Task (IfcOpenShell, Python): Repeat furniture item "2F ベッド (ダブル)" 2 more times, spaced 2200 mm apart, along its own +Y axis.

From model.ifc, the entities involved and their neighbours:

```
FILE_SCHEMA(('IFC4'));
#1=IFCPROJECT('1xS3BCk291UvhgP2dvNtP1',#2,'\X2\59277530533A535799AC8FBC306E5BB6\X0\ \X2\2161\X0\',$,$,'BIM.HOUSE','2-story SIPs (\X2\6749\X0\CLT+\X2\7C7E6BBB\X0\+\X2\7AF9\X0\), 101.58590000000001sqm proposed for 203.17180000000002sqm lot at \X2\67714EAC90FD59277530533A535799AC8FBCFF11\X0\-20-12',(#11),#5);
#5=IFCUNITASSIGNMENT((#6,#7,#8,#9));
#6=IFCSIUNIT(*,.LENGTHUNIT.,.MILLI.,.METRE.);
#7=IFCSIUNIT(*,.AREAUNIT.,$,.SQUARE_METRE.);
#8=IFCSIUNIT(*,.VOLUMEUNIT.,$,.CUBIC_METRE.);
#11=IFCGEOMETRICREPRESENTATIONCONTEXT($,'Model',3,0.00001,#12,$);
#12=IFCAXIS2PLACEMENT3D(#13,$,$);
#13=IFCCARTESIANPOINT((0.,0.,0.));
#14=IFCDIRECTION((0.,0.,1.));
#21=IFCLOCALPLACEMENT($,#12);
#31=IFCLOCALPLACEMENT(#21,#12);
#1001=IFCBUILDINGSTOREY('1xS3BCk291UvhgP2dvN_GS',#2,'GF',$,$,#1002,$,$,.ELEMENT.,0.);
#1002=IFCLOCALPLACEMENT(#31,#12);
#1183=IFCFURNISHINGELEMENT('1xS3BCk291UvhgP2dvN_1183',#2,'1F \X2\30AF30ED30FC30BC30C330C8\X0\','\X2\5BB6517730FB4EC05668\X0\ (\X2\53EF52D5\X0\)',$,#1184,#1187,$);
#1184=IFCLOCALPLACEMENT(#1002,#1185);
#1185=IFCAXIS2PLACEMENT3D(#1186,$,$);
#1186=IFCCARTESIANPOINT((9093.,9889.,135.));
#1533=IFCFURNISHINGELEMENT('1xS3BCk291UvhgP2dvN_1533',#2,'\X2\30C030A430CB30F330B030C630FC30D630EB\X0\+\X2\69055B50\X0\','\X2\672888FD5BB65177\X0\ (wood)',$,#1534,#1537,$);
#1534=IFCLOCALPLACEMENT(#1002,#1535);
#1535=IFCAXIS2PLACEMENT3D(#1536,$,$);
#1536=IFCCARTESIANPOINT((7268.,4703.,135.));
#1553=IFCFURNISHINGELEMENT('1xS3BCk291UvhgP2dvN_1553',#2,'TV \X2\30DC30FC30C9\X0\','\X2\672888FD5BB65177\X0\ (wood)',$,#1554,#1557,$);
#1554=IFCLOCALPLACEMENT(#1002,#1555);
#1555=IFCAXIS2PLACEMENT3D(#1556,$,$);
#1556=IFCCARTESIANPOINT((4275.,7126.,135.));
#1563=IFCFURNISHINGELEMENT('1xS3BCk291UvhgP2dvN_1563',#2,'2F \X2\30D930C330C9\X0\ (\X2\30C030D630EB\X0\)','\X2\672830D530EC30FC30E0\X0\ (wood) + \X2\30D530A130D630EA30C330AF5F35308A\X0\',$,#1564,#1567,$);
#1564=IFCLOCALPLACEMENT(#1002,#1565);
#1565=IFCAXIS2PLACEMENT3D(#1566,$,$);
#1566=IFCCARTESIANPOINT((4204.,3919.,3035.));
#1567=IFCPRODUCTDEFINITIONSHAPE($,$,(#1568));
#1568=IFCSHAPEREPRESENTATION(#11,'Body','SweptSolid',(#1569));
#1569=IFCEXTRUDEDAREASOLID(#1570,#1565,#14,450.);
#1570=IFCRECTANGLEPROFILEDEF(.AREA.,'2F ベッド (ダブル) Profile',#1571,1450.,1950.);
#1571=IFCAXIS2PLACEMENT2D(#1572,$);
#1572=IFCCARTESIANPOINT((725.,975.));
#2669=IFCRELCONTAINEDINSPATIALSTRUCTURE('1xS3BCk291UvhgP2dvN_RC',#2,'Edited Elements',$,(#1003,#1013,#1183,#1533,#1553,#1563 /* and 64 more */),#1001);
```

```python
import ifcopenshell
import ifcopenshell.api.geometry
import ifcopenshell.api.root
import ifcopenshell.util.element
import ifcopenshell.util.placement
import ifcopenshell.util.unit

model = ifcopenshell.open("model.ifc")
unit_scale = ifcopenshell.util.unit.calculate_unit_scale(model)


def reuse_history(source, copy):
    """copy_class also copies each property set's owner history, people and application; keep the originals."""
    for rel in copy.IsDefinedBy:
        if rel.is_a("IfcRelDefinesByProperties") and (history := rel.RelatingPropertyDefinition.OwnerHistory):
            rel.RelatingPropertyDefinition.OwnerHistory = source.OwnerHistory
            ifcopenshell.util.element.remove_deep2(model, history)


source = model.by_id(1563)
base = ifcopenshell.util.placement.get_local_placement(source.ObjectPlacement)
step = base[:3, 1] * 2.2 / unit_scale

for i in range(1, 3):
    copy = ifcopenshell.api.root.copy_class(model, product=source)
    copy.Representation = ifcopenshell.util.element.copy_deep(
        model, source.Representation, exclude=["IfcGeometricRepresentationContext", "IfcRepresentationMap"]
    )
    reuse_history(source, copy)
    matrix = base.copy()
    matrix[:3, 3] += i * step
    print("added at", matrix[:3, 3].round(3) + 0.0)
    ifcopenshell.api.geometry.edit_object_placement(model, product=copy, matrix=matrix, is_si=False)

model.write("model_edited.ifc")
```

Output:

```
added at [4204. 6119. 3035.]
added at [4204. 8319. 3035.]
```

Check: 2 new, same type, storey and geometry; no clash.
